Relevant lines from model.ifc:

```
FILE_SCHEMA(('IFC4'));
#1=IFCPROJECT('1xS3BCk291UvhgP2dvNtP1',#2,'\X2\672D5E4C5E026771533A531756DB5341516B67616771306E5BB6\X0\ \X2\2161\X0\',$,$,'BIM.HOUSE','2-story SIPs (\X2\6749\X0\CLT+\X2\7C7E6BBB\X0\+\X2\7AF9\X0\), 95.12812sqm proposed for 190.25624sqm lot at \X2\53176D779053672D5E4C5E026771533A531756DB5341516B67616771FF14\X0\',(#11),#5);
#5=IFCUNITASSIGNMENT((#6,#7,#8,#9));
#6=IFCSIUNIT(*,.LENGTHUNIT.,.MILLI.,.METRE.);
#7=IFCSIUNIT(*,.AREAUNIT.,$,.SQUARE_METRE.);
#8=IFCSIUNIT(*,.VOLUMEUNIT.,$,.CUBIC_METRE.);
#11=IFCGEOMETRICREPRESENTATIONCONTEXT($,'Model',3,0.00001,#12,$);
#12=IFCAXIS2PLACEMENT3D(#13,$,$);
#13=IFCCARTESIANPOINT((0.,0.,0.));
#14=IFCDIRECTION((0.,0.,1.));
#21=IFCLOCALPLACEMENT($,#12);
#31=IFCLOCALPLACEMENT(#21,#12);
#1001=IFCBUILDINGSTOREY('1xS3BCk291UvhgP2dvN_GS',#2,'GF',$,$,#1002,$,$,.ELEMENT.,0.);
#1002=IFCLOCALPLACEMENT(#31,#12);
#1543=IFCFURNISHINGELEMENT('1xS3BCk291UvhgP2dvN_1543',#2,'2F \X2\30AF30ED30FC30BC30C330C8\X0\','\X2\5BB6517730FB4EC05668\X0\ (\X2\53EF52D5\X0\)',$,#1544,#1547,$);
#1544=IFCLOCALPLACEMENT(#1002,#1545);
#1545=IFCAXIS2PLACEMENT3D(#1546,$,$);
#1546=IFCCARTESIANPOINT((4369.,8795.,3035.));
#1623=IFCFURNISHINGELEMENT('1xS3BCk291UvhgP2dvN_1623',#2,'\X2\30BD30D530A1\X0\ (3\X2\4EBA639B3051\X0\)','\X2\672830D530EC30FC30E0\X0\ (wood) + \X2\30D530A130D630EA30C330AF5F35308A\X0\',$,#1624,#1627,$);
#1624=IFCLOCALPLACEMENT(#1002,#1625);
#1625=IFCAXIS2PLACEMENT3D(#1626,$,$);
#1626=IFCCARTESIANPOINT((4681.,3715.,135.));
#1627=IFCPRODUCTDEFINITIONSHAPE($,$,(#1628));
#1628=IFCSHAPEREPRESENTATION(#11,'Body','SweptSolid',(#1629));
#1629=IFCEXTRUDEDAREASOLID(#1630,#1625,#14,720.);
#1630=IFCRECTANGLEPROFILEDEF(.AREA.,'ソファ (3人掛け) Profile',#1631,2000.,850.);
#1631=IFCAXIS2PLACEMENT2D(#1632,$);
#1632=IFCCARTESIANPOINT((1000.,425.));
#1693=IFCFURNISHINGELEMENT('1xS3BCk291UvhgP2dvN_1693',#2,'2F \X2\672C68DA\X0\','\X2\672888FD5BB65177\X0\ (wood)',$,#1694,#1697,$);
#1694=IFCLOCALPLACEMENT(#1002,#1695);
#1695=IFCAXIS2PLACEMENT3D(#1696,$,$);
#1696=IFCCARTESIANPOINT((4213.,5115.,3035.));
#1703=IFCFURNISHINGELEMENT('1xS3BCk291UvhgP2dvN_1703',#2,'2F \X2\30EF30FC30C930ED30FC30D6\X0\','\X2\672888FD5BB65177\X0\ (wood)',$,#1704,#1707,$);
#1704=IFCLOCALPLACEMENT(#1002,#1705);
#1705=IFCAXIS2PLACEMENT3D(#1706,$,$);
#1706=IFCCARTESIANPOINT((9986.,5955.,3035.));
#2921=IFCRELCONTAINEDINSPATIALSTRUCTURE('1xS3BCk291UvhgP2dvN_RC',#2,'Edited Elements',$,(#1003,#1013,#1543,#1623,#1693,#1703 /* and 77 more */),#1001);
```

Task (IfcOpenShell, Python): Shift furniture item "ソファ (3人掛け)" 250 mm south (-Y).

```python
import ifcopenshell
import ifcopenshell.api.geometry
import ifcopenshell.util.placement

model = ifcopenshell.open("model.ifc")

item = model.by_guid("1xS3BCk291UvhgP2dvN_1623")
matrix = ifcopenshell.util.placement.get_local_placement(item.ObjectPlacement)
matrix[1, 3] -= 250.0
ifcopenshell.api.geometry.edit_object_placement(model, product=item, matrix=matrix, is_si=False)

print(ifcopenshell.util.placement.get_local_placement(item.ObjectPlacement).round(3) + 0.0)

model.write("model-out.ifc")
```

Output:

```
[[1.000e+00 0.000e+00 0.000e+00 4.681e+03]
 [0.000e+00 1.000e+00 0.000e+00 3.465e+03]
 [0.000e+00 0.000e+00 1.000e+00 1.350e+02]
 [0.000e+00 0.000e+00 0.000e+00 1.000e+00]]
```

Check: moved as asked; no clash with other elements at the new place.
